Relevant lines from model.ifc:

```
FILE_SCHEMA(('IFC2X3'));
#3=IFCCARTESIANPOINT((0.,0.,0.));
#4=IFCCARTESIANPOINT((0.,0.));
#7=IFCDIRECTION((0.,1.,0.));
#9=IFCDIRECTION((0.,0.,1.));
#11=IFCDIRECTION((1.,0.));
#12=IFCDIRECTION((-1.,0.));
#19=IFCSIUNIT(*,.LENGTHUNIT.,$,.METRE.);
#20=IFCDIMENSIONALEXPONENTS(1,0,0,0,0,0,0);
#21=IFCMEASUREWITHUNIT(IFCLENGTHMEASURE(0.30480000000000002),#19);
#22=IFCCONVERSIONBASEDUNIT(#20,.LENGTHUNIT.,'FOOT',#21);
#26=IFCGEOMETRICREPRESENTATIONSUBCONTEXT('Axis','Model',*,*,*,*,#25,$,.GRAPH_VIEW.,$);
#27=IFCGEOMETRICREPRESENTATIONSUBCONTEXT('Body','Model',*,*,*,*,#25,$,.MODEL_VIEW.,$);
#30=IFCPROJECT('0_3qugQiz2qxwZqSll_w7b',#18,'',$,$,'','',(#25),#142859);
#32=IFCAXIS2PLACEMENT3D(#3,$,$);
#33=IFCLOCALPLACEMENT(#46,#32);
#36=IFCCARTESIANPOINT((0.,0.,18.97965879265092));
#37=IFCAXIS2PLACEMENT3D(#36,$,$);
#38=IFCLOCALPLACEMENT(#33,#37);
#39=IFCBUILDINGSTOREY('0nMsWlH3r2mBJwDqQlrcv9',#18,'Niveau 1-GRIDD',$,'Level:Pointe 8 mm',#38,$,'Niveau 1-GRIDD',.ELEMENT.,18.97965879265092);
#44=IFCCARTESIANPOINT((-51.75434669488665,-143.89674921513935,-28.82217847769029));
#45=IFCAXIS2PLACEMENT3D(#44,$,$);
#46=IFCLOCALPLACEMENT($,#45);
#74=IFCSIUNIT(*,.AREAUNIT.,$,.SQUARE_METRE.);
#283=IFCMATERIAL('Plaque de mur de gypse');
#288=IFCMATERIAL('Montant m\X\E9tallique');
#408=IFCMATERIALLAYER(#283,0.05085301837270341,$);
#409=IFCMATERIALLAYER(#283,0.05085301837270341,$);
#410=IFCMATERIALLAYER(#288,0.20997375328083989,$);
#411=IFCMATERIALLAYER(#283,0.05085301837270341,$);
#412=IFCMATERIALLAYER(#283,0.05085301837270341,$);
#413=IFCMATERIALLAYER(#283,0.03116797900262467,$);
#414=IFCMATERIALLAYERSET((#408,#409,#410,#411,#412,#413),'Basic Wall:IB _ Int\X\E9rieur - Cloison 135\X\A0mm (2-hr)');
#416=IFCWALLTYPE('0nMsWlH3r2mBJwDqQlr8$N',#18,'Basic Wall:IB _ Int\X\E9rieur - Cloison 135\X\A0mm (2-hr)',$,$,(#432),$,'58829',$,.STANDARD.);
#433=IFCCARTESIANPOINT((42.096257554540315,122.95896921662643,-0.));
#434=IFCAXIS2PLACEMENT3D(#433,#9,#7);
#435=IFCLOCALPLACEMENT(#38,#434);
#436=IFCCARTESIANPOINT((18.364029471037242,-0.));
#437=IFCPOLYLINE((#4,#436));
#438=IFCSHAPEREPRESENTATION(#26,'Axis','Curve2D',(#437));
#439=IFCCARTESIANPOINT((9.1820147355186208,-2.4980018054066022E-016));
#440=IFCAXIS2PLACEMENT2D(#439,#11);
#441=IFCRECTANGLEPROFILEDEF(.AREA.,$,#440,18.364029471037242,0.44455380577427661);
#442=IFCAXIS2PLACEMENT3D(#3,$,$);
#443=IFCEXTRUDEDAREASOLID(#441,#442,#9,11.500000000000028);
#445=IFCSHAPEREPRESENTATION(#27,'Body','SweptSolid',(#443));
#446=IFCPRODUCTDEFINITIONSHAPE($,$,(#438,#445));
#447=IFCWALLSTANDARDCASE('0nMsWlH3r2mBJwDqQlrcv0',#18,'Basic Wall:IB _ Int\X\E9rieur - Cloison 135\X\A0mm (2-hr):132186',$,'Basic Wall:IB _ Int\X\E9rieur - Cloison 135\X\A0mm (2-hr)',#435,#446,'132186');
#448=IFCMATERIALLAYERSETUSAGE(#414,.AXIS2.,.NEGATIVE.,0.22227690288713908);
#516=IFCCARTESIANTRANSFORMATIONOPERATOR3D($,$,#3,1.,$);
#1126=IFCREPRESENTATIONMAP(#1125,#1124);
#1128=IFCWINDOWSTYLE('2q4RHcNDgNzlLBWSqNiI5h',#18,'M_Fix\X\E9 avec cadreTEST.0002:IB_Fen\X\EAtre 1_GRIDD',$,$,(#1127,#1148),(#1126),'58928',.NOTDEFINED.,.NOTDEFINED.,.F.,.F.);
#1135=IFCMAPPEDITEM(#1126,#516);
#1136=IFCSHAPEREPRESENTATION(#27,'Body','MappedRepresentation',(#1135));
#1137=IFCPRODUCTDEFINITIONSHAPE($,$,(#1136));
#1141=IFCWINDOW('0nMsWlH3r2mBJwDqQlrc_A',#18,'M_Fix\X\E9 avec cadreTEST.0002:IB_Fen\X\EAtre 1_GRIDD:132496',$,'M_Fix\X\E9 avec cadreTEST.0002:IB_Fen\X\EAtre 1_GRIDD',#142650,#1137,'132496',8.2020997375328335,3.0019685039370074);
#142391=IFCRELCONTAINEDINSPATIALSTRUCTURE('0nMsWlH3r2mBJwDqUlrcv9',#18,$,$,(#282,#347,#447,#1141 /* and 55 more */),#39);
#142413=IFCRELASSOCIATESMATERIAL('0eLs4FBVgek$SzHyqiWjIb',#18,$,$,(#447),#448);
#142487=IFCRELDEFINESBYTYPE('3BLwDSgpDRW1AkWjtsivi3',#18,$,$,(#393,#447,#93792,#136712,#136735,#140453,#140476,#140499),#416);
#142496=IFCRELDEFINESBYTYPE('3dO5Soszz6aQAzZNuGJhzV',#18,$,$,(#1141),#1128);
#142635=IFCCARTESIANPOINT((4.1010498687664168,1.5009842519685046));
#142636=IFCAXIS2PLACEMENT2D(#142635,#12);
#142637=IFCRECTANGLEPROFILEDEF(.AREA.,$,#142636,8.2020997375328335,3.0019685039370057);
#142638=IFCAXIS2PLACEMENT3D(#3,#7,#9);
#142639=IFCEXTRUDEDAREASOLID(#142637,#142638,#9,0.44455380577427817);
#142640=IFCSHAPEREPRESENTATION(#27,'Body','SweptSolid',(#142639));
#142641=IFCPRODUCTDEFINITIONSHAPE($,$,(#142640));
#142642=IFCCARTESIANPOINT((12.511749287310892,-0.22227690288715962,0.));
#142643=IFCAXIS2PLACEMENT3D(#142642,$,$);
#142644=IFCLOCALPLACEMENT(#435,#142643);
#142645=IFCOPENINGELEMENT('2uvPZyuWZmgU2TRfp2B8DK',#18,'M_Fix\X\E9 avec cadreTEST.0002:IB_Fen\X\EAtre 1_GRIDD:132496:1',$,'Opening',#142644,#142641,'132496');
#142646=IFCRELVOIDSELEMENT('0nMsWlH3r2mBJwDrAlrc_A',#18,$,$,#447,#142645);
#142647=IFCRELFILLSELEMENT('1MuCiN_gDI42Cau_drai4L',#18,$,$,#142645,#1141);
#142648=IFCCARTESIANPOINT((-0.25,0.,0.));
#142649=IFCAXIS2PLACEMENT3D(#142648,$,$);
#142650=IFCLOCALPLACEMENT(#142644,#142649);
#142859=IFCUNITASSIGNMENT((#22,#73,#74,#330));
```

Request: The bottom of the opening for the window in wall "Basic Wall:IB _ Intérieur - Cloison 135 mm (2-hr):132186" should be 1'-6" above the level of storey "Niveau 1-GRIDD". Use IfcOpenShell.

```python
import numpy as np
import ifcopenshell
import ifcopenshell.api.geometry
import ifcopenshell.geom
import ifcopenshell.util.element
import ifcopenshell.util.placement
import ifcopenshell.util.shape
import ifcopenshell.util.unit

model = ifcopenshell.open("model.ifc")
unit_scale = ifcopenshell.util.unit.calculate_unit_scale(model)

window = model.by_guid("0nMsWlH3r2mBJwDqQlrc_A")
opening = window.FillsVoids[0].RelatingOpeningElement
storey = ifcopenshell.util.element.get_container(window, ifc_class="IfcBuildingStorey")
level = ifcopenshell.util.placement.get_local_placement(storey.ObjectPlacement)[2, 3]

# The opening's origin need not be at the sill, so measure its lowest point.
shape = ifcopenshell.geom.create_shape(ifcopenshell.geom.settings(), opening)
bottom = ifcopenshell.util.shape.get_shape_bottom_elevation(shape, shape.geometry) / unit_scale
dz = level + 18 * 0.0254 / unit_scale - bottom

shift = np.array([0.0, 0.0, dz])
# The window is placed relative to its opening, so it follows when the opening moves.
matrix = ifcopenshell.util.placement.get_local_placement(opening.ObjectPlacement)
matrix[:3, 3] += shift
ifcopenshell.api.geometry.edit_object_placement(
    model, product=opening, matrix=matrix, is_si=False, should_transform_children=True
)

print(f"moved by {dz * unit_scale:+.3f} m")

model.write("model_edited.ifc")
```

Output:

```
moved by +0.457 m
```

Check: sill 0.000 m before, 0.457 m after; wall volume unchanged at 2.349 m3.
